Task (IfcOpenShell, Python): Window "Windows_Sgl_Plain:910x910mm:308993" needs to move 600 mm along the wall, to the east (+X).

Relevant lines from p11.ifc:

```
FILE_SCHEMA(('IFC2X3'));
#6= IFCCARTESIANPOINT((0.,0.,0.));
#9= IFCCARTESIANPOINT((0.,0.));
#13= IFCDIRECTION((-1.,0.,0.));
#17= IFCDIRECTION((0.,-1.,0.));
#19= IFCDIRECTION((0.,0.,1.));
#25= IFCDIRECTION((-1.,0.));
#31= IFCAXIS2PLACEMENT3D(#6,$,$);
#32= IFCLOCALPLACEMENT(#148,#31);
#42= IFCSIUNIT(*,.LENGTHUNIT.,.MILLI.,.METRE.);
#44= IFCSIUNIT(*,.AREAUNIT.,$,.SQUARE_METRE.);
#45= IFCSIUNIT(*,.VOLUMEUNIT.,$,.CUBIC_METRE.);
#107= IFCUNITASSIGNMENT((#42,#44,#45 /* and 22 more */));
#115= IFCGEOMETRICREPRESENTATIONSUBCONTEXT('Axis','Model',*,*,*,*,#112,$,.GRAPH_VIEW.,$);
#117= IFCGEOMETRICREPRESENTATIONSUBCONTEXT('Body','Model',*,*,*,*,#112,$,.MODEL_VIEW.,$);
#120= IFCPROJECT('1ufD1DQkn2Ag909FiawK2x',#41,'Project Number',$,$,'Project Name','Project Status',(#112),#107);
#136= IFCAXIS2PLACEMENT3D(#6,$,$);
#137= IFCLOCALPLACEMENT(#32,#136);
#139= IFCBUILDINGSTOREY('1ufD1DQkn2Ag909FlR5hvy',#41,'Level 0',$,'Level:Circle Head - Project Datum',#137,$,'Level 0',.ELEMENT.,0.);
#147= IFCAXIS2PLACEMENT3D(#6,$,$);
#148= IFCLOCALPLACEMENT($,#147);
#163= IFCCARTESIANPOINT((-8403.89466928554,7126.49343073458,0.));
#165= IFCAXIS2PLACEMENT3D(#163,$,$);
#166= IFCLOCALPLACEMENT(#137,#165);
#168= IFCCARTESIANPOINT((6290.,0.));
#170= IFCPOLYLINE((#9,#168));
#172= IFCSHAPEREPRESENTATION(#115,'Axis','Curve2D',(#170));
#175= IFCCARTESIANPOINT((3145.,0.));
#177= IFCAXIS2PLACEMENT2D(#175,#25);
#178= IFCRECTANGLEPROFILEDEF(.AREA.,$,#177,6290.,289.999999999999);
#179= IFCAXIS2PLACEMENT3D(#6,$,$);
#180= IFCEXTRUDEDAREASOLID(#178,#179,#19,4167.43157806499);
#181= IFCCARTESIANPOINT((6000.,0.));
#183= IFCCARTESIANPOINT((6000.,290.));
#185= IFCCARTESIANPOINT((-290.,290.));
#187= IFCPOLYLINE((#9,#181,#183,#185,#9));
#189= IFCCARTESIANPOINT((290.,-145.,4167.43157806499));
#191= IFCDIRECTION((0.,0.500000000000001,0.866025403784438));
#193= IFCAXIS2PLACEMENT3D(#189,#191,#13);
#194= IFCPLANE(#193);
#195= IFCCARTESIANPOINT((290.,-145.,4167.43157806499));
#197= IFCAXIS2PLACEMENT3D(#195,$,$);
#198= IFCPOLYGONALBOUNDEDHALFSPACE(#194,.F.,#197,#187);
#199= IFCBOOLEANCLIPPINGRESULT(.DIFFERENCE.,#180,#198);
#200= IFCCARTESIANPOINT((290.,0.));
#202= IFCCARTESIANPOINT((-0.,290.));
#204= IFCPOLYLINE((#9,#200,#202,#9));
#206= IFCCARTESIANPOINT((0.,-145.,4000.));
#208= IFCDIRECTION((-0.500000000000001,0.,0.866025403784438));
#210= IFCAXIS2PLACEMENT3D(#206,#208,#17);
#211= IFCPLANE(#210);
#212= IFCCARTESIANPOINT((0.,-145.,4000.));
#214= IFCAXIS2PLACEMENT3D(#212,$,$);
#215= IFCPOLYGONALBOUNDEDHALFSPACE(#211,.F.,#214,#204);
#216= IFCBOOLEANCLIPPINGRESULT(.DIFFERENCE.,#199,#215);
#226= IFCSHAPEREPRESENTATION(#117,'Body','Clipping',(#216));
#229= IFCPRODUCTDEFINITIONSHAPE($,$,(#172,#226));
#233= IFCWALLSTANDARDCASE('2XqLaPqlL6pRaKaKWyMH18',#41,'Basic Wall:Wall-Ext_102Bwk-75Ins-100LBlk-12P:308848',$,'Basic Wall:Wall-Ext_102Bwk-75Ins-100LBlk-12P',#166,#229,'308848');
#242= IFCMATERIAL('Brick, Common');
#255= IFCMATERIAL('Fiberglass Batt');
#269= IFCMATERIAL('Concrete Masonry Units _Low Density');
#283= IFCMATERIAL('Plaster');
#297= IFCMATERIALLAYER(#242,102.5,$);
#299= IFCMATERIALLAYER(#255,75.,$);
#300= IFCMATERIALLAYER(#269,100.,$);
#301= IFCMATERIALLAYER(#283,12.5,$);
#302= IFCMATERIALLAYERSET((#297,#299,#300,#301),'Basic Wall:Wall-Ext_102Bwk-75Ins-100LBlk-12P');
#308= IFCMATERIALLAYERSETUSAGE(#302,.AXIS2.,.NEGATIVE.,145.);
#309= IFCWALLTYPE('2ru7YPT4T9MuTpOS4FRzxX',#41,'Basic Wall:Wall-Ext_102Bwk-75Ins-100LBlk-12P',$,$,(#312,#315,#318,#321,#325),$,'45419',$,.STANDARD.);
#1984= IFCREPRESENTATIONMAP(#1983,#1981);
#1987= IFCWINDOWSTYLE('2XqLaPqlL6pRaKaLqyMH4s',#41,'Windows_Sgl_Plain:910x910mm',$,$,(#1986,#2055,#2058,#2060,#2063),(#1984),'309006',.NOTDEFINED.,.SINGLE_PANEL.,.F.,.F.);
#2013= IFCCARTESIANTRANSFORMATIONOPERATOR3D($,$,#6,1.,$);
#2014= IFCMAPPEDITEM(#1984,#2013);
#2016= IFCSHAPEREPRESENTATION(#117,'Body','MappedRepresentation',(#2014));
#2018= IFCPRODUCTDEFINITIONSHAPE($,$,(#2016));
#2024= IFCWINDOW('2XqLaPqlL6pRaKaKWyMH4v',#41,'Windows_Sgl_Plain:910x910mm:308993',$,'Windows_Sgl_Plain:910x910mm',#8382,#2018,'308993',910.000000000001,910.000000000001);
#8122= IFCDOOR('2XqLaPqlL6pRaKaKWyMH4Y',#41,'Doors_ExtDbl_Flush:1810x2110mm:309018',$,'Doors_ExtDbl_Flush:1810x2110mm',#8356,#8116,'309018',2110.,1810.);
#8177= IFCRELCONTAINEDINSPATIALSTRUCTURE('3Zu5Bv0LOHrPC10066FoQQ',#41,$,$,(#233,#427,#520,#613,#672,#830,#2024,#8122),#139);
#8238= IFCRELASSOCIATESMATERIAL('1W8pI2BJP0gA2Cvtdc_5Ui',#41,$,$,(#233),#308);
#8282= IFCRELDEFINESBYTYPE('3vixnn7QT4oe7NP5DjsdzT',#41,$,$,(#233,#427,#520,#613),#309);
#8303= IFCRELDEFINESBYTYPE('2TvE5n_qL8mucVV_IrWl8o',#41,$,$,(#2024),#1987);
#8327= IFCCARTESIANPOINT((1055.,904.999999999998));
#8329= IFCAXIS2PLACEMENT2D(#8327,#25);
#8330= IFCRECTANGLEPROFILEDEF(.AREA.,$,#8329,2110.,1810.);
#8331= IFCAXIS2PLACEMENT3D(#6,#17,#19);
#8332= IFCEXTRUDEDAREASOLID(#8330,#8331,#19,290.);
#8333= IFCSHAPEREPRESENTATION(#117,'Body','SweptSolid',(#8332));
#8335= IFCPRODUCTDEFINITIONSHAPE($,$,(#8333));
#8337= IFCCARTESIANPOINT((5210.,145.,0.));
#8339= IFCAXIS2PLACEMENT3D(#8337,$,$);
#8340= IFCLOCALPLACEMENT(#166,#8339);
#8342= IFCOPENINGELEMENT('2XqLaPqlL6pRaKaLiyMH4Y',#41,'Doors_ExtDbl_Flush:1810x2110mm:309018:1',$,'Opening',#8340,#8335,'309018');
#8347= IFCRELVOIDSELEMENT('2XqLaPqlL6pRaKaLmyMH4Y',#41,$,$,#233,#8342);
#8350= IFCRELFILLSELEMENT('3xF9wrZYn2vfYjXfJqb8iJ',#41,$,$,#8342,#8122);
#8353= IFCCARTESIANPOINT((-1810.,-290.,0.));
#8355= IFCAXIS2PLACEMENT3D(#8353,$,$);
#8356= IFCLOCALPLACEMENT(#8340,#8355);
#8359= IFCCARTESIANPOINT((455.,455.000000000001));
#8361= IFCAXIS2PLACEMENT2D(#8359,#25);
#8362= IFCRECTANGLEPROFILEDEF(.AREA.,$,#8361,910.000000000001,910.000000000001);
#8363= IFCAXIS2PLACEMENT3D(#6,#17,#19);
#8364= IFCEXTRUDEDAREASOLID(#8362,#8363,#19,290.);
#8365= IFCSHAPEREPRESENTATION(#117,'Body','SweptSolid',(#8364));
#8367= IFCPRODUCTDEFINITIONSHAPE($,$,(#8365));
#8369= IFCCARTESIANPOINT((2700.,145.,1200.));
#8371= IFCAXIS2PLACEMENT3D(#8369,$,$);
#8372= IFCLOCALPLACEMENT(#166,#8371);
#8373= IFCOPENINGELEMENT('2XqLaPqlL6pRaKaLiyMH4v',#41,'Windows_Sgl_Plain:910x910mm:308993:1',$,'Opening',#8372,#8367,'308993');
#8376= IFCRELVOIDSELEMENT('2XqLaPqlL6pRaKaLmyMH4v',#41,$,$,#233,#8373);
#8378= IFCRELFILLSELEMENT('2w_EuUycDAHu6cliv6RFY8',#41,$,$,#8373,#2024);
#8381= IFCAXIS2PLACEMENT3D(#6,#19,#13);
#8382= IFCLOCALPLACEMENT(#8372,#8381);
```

```python
import ifcopenshell
import ifcopenshell.api.geometry
import ifcopenshell.util.placement
import ifcopenshell.util.unit

model = ifcopenshell.open("p11.ifc")
unit_scale = ifcopenshell.util.unit.calculate_unit_scale(model)

window = model.by_guid("2XqLaPqlL6pRaKaKWyMH4v")
opening = window.FillsVoids[0].RelatingOpeningElement
wall = opening.VoidsElements[0].RelatingBuildingElement

wall_matrix = ifcopenshell.util.placement.get_local_placement(wall.ObjectPlacement)
shift = wall_matrix[:3, 0] * 0.6 / unit_scale
before = ifcopenshell.util.placement.get_local_placement(window.ObjectPlacement)[:3, 3].copy()

# The window is placed relative to its opening, so it follows when the opening moves.
matrix = ifcopenshell.util.placement.get_local_placement(opening.ObjectPlacement)
matrix[:3, 3] += shift
ifcopenshell.api.geometry.edit_object_placement(
    model, product=opening, matrix=matrix, is_si=False, should_transform_children=True
)

after = ifcopenshell.util.placement.get_local_placement(window.ObjectPlacement)[:3, 3]
print("window moved by", (after - before).round(3) + 0.0)

model.write("p11_edited.ifc")
```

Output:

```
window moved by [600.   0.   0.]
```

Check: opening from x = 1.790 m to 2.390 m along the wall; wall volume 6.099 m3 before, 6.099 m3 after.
